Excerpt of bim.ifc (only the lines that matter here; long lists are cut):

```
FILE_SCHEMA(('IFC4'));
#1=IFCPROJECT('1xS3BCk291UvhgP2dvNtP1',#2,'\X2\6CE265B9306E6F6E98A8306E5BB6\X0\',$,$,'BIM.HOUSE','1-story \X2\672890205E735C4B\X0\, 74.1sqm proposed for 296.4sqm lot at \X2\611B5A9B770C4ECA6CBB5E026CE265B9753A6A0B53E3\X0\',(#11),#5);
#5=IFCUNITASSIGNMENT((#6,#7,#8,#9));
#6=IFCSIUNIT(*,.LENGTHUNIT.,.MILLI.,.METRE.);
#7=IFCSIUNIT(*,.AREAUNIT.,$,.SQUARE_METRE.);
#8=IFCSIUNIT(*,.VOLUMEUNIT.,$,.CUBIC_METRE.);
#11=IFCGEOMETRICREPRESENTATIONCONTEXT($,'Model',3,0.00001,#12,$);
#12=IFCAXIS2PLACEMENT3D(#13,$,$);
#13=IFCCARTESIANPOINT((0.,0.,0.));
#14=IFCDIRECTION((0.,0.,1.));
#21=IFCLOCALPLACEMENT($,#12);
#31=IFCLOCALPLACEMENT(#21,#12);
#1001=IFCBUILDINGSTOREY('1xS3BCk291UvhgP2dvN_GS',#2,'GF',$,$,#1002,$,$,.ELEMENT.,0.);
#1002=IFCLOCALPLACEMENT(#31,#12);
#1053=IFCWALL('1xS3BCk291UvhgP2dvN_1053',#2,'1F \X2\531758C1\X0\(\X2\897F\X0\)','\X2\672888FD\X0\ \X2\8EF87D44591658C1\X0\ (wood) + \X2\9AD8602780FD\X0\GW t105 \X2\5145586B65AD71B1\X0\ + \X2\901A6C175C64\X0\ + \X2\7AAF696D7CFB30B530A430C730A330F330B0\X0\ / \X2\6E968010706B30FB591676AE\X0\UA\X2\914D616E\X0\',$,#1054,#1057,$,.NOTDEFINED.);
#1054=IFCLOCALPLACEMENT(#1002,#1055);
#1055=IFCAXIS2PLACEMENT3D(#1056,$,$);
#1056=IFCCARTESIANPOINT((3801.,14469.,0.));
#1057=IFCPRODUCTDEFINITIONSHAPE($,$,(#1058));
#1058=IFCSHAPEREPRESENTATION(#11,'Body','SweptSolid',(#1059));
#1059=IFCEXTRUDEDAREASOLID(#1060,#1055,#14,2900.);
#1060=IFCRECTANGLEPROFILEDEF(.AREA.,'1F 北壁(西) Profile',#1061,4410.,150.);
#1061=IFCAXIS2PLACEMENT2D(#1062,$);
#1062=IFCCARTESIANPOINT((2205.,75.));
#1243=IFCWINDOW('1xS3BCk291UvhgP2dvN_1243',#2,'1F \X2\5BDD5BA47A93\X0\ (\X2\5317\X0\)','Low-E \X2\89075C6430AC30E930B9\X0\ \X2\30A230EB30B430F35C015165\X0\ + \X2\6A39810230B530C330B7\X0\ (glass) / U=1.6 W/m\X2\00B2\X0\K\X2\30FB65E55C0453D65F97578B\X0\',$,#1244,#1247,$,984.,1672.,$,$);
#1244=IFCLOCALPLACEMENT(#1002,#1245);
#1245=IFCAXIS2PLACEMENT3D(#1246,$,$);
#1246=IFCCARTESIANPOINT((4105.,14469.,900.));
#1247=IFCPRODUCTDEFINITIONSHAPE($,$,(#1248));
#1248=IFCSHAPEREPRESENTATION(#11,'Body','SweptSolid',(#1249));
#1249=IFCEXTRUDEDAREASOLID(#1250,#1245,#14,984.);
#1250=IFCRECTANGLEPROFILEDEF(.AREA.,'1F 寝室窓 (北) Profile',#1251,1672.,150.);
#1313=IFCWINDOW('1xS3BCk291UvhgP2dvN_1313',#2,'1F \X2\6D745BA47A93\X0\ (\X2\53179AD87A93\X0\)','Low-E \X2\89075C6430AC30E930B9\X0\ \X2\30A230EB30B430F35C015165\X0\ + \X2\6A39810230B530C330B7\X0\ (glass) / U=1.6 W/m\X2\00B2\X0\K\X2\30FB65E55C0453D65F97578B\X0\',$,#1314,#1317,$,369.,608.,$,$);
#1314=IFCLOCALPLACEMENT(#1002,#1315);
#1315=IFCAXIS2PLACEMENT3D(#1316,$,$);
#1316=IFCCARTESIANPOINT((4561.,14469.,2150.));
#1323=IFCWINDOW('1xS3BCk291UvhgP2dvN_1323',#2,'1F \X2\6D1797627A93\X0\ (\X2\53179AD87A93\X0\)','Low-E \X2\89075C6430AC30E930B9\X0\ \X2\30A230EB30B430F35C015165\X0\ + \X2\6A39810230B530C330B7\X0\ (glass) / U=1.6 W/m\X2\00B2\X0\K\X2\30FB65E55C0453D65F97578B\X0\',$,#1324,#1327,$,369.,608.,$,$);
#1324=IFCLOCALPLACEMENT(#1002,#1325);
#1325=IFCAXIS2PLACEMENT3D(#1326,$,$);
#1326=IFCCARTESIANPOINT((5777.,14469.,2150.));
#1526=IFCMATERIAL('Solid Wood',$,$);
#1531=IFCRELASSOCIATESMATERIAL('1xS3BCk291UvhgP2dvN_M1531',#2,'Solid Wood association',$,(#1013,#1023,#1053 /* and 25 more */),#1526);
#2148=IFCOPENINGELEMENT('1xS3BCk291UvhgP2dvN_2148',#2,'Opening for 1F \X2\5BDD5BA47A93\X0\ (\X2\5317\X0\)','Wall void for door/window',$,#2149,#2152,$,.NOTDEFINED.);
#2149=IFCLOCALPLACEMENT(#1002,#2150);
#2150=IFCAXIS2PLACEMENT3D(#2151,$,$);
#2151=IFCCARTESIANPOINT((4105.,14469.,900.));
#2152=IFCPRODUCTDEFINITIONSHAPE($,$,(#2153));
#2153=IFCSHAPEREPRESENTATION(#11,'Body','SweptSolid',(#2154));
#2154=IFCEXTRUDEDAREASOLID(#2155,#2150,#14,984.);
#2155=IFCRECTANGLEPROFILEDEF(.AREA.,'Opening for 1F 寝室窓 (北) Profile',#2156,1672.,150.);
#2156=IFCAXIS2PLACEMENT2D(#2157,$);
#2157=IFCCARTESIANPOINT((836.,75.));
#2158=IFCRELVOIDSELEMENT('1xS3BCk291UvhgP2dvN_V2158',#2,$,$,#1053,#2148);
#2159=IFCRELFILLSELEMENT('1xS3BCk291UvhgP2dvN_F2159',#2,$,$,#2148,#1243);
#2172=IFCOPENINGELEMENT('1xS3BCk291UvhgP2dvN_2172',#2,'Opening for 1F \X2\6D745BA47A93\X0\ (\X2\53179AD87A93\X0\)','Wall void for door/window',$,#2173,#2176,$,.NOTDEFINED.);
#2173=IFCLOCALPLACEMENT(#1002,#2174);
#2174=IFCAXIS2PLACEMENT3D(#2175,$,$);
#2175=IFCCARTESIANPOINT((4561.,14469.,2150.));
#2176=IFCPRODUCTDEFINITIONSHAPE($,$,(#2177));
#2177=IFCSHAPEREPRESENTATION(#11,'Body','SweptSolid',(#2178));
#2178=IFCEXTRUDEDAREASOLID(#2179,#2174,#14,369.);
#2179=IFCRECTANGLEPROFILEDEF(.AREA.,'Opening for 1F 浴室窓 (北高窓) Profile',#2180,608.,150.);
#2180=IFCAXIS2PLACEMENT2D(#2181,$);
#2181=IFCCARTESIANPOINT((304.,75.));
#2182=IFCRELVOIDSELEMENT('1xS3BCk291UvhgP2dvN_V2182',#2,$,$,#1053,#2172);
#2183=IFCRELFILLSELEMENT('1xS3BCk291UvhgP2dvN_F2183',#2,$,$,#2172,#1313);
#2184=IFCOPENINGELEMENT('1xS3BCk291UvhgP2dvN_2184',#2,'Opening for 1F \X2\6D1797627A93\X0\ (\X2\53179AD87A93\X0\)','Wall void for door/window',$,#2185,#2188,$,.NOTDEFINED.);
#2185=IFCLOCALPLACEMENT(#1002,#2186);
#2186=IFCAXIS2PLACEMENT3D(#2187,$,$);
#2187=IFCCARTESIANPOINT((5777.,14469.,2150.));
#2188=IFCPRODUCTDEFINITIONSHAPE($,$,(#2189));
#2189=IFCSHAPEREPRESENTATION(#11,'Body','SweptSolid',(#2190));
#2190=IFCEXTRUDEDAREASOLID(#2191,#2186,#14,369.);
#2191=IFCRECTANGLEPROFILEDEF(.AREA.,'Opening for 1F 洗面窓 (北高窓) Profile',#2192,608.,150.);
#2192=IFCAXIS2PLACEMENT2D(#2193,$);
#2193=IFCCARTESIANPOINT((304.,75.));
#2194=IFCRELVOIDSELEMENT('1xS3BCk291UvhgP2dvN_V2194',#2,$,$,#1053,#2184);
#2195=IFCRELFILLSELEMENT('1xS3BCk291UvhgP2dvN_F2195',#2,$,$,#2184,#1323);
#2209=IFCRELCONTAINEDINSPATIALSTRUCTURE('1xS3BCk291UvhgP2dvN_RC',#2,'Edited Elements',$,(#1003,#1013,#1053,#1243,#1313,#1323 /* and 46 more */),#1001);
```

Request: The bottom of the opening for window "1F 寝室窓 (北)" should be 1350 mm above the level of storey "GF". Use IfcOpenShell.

```python
import numpy as np
import ifcopenshell
import ifcopenshell.api.geometry
import ifcopenshell.geom
import ifcopenshell.util.element
import ifcopenshell.util.placement
import ifcopenshell.util.shape
import ifcopenshell.util.unit

model = ifcopenshell.open("bim.ifc")
unit_scale = ifcopenshell.util.unit.calculate_unit_scale(model)

window = model.by_guid("1xS3BCk291UvhgP2dvN_1243")
opening = window.FillsVoids[0].RelatingOpeningElement
storey = ifcopenshell.util.element.get_container(window, ifc_class="IfcBuildingStorey")
level = ifcopenshell.util.placement.get_local_placement(storey.ObjectPlacement)[2, 3]

# The opening's origin need not be at the sill, so measure its lowest point.
shape = ifcopenshell.geom.create_shape(ifcopenshell.geom.settings(), opening)
bottom = ifcopenshell.util.shape.get_shape_bottom_elevation(shape, shape.geometry) / unit_scale
dz = level + 1.35 / unit_scale - bottom

shift = np.array([0.0, 0.0, dz])
# The window is not placed relative to its opening, so move both.
for product in (opening, window):
    matrix = ifcopenshell.util.placement.get_local_placement(product.ObjectPlacement)
    matrix[:3, 3] += shift
    ifcopenshell.api.geometry.edit_object_placement(model, product=product, matrix=matrix, is_si=False)

print(f"moved by {dz * unit_scale:+.3f} m")

model.write("bim_v2.ifc")
```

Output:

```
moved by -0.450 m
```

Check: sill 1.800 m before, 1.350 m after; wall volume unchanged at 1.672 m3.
